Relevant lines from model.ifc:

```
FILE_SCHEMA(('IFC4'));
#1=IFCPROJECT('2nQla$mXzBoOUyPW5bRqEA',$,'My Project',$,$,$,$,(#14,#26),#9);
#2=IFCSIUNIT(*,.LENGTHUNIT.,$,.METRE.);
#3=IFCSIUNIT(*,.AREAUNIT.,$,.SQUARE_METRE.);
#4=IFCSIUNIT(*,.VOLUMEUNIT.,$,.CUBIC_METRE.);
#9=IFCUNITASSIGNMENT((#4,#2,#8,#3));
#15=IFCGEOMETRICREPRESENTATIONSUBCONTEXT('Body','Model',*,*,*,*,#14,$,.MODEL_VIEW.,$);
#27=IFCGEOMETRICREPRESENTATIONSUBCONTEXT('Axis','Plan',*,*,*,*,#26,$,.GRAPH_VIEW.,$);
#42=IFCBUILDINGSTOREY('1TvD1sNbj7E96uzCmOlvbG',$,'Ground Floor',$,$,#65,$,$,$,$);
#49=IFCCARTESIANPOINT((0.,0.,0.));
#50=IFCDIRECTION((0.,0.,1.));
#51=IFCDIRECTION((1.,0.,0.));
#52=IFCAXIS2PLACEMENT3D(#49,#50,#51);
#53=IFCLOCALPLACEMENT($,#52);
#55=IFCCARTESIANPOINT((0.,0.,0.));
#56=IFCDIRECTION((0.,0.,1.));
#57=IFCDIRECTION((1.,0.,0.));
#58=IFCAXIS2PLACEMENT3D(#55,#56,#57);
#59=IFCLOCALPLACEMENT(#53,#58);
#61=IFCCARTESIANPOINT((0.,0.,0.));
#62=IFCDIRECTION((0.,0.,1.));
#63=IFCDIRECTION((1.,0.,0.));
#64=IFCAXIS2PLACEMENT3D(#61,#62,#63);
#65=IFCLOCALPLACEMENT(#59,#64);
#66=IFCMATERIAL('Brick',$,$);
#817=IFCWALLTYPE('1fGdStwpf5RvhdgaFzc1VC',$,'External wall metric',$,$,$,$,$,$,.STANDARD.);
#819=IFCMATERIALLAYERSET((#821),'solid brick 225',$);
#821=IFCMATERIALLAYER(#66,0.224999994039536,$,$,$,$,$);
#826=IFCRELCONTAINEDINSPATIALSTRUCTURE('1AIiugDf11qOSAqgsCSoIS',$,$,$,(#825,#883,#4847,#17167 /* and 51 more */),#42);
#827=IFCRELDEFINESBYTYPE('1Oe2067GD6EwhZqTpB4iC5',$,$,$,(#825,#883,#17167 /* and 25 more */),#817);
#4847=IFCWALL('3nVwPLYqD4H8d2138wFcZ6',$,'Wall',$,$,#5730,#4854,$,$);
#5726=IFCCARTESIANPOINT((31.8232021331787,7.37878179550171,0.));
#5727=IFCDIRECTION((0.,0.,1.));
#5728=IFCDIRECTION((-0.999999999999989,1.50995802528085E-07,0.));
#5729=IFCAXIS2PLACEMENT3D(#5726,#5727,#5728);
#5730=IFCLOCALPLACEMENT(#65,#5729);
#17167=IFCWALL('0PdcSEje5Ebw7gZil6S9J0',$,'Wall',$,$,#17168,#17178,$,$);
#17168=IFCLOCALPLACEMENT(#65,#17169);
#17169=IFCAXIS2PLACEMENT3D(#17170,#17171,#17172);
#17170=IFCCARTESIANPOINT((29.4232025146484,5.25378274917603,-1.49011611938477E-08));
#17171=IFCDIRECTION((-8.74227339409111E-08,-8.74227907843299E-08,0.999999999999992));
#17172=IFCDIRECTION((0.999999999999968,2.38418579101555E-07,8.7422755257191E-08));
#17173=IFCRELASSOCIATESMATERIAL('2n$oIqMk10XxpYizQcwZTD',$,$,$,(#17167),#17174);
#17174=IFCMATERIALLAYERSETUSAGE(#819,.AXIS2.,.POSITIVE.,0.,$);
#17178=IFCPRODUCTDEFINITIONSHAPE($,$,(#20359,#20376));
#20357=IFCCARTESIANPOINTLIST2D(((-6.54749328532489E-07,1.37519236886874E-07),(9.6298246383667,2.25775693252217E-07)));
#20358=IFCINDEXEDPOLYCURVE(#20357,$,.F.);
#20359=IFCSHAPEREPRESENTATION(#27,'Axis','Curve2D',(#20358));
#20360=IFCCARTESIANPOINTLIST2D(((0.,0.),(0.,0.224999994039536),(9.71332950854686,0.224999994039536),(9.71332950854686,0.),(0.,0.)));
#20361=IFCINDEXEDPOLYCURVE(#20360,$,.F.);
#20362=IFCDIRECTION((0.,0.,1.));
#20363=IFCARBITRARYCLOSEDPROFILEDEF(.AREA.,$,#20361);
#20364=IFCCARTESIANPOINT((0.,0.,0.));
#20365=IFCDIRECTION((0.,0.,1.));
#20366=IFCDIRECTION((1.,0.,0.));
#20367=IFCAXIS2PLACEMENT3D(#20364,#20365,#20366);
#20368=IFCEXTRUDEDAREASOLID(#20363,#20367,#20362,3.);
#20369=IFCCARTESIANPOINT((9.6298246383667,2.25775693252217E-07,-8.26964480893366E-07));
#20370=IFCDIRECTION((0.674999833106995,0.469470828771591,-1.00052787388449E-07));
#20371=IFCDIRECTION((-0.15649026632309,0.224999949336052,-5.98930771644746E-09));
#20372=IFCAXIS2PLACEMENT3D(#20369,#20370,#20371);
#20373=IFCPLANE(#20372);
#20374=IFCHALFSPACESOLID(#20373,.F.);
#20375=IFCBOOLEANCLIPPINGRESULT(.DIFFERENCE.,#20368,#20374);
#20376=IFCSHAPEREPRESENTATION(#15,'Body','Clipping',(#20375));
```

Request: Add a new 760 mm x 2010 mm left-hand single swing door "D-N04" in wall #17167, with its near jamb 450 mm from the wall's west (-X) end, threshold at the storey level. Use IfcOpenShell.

```python
import numpy as np
import ifcopenshell
import ifcopenshell.api.feature
import ifcopenshell.api.geometry
import ifcopenshell.api.root
import ifcopenshell.api.spatial
import ifcopenshell.geom
import ifcopenshell.util.element
import ifcopenshell.util.placement
import ifcopenshell.util.representation
import ifcopenshell.util.shape
import ifcopenshell.util.unit

model = ifcopenshell.open("model.ifc")
unit_scale = ifcopenshell.util.unit.calculate_unit_scale(model)
settings = ifcopenshell.geom.settings()


def volume(element):
    """Net volume in cubic metres, openings subtracted."""
    shape = ifcopenshell.geom.create_shape(settings, element)
    return ifcopenshell.util.shape.get_volume(shape.geometry)


wall = model.by_guid("0PdcSEje5Ebw7gZil6S9J0")
storey = ifcopenshell.util.element.get_container(wall, ifc_class="IfcBuildingStorey")
context = ifcopenshell.util.representation.get_context(model, "Model", "Body", "MODEL_VIEW")
before = volume(wall)

width, height, from_end, sill = 0.76, 2.01, 0.45, 0.0  # metres

# The wall runs along its own X axis, and the end named is its -X end.
wall_shape = ifcopenshell.geom.create_shape(settings, wall)
x, y, z = ifcopenshell.util.shape.get_vertices(wall_shape.geometry).T
start = x.min() + from_end
face, thickness = float(y.min()), float(y.max() - y.min())
wall_matrix = ifcopenshell.util.placement.get_local_placement(wall.ObjectPlacement)
level = ifcopenshell.util.placement.get_local_placement(storey.ObjectPlacement)[2, 3]


def in_wall(x, y):
    """Placement at x, y metres in the wall's axes, at sill height."""
    matrix = wall_matrix.copy()
    matrix[:, 3] = wall_matrix @ np.array([x / unit_scale, y / unit_scale, 0.0, 1.0])
    matrix[2, 3] = level + sill / unit_scale
    return matrix


# Opening: a box that overshoots both wall faces by 50 mm.
opening = ifcopenshell.api.root.create_entity(model, ifc_class="IfcOpeningElement", predefined_type="OPENING")
box = ifcopenshell.api.geometry.add_wall_representation(
    model, context=context, length=width, height=height, thickness=thickness + 0.1
)
ifcopenshell.api.geometry.assign_representation(model, product=opening, representation=box)
ifcopenshell.api.geometry.edit_object_placement(model, product=opening, matrix=in_wall(start, face - 0.05), is_si=False)
ifcopenshell.api.feature.add_feature(model, feature=opening, element=wall)

door = ifcopenshell.api.root.create_entity(model, ifc_class="IfcDoor", name="D-N04", predefined_type="DOOR")
door.OverallWidth, door.OverallHeight = width / unit_scale, height / unit_scale
door.OperationType = "SINGLE_SWING_LEFT"
body = ifcopenshell.api.geometry.add_door_representation(
    model,
    context=context,
    overall_width=door.OverallWidth,
    overall_height=door.OverallHeight,
    operation_type="SINGLE_SWING_LEFT",
    lining_properties={"LiningDepth": thickness / unit_scale, "ThresholdDepth": thickness / unit_scale},
)
ifcopenshell.api.geometry.assign_representation(model, product=door, representation=body)
ifcopenshell.api.spatial.assign_container(model, products=[door], relating_structure=storey)
ifcopenshell.api.feature.add_filling(model, opening=opening, element=door)

# The lining spans the wall, so the door starts at the wall face.
ifcopenshell.api.geometry.edit_object_placement(model, product=door, matrix=in_wall(start, face), is_si=False)

after = volume(wall)

print(f"wall volume {before:.3f} -> {after:.3f} m3")

model.write("model-out.ifc")
```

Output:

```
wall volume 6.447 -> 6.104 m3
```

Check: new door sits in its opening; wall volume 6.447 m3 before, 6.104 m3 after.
